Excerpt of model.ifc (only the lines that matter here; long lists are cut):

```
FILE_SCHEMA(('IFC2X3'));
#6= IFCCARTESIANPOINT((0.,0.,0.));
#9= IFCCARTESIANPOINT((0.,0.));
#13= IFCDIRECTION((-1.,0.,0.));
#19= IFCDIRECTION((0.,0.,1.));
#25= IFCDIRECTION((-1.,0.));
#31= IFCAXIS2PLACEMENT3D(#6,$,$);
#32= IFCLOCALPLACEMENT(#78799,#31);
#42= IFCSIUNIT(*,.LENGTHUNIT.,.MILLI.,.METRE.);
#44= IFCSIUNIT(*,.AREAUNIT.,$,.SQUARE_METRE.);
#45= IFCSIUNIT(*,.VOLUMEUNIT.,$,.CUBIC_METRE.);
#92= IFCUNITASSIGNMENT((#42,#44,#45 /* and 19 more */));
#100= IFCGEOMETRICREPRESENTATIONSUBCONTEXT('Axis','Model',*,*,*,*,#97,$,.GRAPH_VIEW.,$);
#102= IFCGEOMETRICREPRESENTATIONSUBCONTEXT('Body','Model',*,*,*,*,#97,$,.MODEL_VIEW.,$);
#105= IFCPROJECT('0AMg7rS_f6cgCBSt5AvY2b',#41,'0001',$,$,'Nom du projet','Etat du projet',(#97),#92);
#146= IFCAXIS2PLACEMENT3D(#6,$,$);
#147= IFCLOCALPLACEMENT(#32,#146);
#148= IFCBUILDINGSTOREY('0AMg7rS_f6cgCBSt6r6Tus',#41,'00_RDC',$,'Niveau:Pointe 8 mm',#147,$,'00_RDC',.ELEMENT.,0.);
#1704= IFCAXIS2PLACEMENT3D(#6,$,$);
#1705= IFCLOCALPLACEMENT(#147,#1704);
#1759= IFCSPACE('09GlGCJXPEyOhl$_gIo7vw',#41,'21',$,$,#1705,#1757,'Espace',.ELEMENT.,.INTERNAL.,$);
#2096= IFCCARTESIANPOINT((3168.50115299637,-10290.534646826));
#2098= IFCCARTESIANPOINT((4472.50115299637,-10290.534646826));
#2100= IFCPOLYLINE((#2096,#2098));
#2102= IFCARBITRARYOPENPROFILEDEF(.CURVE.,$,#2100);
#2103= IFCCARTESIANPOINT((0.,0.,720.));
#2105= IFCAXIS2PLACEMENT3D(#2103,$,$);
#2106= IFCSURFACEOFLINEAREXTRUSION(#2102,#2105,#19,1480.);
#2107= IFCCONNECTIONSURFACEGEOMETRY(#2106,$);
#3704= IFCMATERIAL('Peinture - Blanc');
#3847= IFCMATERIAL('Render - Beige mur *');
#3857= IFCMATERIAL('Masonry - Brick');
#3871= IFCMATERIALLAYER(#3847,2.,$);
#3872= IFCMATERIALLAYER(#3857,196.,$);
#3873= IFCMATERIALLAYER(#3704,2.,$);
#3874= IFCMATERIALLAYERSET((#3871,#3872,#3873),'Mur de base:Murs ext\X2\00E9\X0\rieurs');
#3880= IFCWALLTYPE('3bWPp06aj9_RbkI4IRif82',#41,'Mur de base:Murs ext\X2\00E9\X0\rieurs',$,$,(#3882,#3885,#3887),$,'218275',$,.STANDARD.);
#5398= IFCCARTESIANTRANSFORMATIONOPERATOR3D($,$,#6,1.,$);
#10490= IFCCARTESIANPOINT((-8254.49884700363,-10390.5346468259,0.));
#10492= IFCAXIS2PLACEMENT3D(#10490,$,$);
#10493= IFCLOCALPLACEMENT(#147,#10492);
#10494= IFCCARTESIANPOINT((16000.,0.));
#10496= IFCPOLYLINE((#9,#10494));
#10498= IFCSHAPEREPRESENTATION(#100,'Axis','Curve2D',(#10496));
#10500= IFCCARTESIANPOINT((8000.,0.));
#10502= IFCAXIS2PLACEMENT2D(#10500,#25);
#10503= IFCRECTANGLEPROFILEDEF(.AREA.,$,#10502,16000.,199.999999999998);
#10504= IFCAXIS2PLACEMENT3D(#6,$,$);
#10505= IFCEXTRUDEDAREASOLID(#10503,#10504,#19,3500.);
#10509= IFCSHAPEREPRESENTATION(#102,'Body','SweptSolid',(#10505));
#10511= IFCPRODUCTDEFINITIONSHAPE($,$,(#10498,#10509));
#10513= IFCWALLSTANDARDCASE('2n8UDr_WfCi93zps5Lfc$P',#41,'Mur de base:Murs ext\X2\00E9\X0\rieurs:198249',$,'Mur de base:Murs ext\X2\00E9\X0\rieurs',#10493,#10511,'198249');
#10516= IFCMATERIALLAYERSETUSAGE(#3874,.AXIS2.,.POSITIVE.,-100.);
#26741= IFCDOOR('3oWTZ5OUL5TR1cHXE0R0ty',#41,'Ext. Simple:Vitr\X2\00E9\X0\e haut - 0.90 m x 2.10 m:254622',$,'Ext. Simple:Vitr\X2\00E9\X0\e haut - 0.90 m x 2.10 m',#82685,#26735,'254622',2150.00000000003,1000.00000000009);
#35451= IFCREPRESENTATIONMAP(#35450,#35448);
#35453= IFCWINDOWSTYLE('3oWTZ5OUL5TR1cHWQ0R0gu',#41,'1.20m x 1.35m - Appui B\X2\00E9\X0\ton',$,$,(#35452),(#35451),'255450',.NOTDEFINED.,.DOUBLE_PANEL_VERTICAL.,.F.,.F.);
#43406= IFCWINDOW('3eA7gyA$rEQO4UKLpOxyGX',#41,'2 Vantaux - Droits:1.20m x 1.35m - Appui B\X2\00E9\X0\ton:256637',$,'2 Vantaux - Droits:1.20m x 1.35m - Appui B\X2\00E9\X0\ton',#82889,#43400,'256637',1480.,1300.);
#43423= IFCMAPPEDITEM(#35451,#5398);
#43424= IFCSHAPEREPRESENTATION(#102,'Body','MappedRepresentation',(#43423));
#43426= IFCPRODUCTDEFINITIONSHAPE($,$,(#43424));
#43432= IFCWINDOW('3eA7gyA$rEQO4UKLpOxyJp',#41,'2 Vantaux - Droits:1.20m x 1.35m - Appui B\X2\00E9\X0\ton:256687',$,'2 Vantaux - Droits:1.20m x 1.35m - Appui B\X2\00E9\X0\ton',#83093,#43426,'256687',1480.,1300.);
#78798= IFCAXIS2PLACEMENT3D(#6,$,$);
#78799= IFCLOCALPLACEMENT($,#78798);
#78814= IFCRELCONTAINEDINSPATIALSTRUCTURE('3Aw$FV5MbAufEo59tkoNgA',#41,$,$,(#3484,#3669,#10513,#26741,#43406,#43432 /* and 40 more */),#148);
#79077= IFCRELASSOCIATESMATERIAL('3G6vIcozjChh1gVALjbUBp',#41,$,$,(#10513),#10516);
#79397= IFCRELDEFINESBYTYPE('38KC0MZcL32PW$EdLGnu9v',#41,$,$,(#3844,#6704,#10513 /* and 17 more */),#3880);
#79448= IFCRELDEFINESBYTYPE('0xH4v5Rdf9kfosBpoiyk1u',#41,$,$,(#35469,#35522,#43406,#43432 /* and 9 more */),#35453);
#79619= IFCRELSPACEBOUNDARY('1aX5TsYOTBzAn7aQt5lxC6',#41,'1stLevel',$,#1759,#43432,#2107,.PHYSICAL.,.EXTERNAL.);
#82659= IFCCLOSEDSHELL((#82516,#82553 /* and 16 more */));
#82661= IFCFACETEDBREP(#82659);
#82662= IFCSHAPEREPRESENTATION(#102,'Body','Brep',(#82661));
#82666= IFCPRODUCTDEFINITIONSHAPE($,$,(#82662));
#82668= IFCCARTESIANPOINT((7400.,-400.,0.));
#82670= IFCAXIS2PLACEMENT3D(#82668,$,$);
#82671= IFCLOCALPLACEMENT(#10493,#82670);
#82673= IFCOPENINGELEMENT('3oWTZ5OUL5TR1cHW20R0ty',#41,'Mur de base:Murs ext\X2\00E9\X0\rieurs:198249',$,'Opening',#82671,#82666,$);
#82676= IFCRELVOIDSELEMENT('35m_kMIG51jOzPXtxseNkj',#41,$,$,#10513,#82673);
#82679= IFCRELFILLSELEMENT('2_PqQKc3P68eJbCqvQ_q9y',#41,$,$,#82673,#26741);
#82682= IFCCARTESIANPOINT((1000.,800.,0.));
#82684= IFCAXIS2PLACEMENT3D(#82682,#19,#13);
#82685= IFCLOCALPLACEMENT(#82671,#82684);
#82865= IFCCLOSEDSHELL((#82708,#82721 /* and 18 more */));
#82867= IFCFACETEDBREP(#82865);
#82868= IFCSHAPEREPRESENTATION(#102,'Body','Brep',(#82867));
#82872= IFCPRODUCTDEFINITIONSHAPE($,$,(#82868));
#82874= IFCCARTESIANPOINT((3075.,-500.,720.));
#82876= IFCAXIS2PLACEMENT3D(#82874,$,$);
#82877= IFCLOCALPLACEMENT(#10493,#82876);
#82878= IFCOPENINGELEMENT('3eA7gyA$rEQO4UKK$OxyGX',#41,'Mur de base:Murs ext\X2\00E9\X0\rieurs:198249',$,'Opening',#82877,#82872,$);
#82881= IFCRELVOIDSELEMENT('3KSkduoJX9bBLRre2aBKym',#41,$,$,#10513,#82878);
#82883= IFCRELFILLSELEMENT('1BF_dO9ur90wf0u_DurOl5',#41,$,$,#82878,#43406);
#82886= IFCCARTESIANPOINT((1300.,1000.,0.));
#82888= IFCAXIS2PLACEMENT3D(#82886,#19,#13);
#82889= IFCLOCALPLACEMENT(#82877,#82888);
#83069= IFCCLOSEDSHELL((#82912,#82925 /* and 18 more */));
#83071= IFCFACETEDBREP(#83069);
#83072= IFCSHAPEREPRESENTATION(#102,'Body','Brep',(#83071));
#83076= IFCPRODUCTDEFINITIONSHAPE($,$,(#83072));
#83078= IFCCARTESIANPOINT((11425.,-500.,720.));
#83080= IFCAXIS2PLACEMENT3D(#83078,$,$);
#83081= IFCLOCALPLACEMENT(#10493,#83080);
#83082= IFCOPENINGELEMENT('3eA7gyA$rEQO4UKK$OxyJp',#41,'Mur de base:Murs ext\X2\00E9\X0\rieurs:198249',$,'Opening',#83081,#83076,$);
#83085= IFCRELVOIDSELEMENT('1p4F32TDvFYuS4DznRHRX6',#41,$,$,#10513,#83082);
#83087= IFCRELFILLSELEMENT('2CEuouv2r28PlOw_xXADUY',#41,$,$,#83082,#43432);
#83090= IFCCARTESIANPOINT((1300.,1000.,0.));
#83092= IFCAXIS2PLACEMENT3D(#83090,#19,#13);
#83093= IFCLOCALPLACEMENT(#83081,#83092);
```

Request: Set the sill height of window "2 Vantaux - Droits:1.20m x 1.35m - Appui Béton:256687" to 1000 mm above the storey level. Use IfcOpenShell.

```python
import numpy as np
import ifcopenshell
import ifcopenshell.api.geometry
import ifcopenshell.geom
import ifcopenshell.util.element
import ifcopenshell.util.placement
import ifcopenshell.util.shape
import ifcopenshell.util.unit

model = ifcopenshell.open("model.ifc")
unit_scale = ifcopenshell.util.unit.calculate_unit_scale(model)

window = model.by_guid("3eA7gyA$rEQO4UKLpOxyJp")
opening = window.FillsVoids[0].RelatingOpeningElement
storey = ifcopenshell.util.element.get_container(window, ifc_class="IfcBuildingStorey")
level = ifcopenshell.util.placement.get_local_placement(storey.ObjectPlacement)[2, 3]

# The opening's origin need not be at the sill, so measure its lowest point.
shape = ifcopenshell.geom.create_shape(ifcopenshell.geom.settings(), opening)
bottom = ifcopenshell.util.shape.get_shape_bottom_elevation(shape, shape.geometry) / unit_scale
dz = level + 1 / unit_scale - bottom

shift = np.array([0.0, 0.0, dz])
# The window is placed relative to its opening, so it follows when the opening moves.
matrix = ifcopenshell.util.placement.get_local_placement(opening.ObjectPlacement)
matrix[:3, 3] += shift
ifcopenshell.api.geometry.edit_object_placement(
    model, product=opening, matrix=matrix, is_si=False, should_transform_children=True
)

# Space boundary surfaces are stored in each space's coordinates; move them too.
for rel in window.ProvidesBoundaries:
    if not rel.ConnectionGeometry:
        continue
    surface = rel.ConnectionGeometry.SurfaceOnRelatingElement
    space_matrix = ifcopenshell.util.placement.get_local_placement(rel.RelatingSpace.ObjectPlacement)
    point = np.array(surface.Position.Location.Coordinates) + space_matrix[:3, :3].T @ shift
    surface.Position = model.createIfcAxis2Placement3D(
        model.createIfcCartesianPoint(point.tolist()), surface.Position.Axis, surface.Position.RefDirection
    )

print(f"moved by {dz * unit_scale:+.3f} m")

model.write("model_rev.ifc")
```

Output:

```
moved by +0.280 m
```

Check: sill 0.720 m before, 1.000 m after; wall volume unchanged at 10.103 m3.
